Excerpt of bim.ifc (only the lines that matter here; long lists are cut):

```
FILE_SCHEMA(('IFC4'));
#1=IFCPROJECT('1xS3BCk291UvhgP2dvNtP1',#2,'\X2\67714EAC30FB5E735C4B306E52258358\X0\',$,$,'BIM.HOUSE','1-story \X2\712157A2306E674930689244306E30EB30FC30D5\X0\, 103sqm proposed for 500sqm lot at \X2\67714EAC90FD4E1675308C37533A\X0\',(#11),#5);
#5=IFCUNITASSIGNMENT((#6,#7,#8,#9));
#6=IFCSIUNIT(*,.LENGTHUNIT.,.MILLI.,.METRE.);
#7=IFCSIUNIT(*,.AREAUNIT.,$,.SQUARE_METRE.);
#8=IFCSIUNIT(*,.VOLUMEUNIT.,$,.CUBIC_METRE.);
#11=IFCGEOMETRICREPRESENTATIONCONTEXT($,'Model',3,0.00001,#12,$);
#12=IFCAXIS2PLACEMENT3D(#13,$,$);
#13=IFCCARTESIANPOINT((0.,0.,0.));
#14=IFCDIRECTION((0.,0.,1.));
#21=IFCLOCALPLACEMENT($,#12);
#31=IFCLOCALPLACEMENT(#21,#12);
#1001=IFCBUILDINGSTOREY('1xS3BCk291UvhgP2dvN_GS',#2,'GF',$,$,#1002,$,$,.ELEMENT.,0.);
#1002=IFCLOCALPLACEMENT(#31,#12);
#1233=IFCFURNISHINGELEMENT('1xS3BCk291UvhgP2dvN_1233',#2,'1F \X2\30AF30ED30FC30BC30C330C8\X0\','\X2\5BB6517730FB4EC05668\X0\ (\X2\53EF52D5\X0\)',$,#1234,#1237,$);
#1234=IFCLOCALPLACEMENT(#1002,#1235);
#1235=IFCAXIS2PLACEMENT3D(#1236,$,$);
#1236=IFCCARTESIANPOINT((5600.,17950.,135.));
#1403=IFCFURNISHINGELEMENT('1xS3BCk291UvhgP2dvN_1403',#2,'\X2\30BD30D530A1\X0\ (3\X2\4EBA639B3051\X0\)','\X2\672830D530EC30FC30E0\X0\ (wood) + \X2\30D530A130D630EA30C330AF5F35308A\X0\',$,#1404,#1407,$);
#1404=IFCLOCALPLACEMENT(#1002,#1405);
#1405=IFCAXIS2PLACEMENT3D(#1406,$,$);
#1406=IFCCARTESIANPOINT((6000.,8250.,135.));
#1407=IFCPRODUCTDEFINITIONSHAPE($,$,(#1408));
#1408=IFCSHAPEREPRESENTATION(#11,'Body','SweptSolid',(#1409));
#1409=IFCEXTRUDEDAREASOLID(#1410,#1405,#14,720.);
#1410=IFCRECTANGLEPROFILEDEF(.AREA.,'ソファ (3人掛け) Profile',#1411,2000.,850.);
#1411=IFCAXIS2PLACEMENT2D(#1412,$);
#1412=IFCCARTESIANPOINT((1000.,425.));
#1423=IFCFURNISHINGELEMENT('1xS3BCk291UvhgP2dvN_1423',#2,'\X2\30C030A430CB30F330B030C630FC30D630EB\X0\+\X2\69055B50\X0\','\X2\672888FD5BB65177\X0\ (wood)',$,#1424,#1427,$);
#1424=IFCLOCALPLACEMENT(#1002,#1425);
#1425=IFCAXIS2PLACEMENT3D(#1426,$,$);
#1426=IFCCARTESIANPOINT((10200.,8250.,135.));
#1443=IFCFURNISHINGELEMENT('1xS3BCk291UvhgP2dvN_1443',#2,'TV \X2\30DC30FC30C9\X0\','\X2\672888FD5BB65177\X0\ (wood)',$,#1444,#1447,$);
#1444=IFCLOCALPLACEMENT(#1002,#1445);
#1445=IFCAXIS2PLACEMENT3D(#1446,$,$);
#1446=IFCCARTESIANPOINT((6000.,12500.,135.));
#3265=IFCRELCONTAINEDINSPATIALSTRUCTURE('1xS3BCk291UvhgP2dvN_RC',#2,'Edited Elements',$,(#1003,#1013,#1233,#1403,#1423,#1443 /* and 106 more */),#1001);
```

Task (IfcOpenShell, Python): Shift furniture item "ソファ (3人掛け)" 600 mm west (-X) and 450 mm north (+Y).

```python
import ifcopenshell
import ifcopenshell.api.geometry
import ifcopenshell.util.placement
import ifcopenshell.util.unit

model = ifcopenshell.open("bim.ifc")
unit_scale = ifcopenshell.util.unit.calculate_unit_scale(model)

item = model.by_guid("1xS3BCk291UvhgP2dvN_1403")
matrix = ifcopenshell.util.placement.get_local_placement(item.ObjectPlacement)
matrix[0, 3] -= 0.6 / unit_scale
matrix[1, 3] += 0.45 / unit_scale
ifcopenshell.api.geometry.edit_object_placement(model, product=item, matrix=matrix, is_si=False)

print(ifcopenshell.util.placement.get_local_placement(item.ObjectPlacement).round(3) + 0.0)

model.write("bim_rev.ifc")
```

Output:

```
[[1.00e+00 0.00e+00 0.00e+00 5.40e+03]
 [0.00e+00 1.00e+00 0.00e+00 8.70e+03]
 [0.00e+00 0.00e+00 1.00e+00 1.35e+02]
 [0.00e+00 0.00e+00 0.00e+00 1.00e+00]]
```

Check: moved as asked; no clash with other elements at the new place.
